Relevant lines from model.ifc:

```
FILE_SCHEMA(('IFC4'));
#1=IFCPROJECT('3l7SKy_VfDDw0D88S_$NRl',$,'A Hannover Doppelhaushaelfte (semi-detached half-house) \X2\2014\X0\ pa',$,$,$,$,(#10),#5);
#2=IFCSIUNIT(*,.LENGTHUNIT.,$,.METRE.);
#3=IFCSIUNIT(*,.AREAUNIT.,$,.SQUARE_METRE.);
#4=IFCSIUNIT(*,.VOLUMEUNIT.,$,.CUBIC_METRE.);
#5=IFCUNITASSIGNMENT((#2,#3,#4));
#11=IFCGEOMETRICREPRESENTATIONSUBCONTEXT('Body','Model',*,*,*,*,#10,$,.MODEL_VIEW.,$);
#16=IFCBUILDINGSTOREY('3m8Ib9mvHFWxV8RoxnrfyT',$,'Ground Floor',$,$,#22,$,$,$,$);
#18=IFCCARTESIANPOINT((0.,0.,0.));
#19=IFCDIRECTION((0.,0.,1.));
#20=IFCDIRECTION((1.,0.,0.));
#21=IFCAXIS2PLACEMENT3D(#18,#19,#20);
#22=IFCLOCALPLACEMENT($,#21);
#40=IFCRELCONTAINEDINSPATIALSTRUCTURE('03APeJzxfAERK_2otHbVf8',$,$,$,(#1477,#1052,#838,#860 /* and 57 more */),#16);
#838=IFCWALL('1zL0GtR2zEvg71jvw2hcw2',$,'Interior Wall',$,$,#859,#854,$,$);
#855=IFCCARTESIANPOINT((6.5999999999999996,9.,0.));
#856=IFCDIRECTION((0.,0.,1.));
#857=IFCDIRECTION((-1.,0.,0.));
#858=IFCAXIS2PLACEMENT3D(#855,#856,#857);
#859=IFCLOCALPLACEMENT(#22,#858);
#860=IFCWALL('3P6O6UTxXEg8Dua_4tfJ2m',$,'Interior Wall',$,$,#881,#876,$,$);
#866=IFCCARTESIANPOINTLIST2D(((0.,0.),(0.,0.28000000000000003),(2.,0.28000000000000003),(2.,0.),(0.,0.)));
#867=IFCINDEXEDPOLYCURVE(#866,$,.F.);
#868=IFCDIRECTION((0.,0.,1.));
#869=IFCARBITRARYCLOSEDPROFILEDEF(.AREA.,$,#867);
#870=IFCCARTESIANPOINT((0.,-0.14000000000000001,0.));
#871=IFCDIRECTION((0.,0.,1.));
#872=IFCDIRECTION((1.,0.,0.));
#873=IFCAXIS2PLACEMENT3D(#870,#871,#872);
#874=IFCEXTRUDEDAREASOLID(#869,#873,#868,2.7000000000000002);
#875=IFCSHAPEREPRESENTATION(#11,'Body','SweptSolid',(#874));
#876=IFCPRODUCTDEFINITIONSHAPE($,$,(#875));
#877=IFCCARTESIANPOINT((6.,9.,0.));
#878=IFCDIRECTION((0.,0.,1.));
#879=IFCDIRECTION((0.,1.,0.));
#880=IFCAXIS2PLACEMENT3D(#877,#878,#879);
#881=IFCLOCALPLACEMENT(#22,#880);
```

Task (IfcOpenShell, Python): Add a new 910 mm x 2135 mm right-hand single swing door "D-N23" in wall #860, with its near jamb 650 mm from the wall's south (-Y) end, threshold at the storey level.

```python
import numpy as np
import ifcopenshell
import ifcopenshell.api.feature
import ifcopenshell.api.geometry
import ifcopenshell.api.root
import ifcopenshell.api.spatial
import ifcopenshell.geom
import ifcopenshell.util.element
import ifcopenshell.util.placement
import ifcopenshell.util.representation
import ifcopenshell.util.shape
import ifcopenshell.util.unit

model = ifcopenshell.open("model.ifc")
unit_scale = ifcopenshell.util.unit.calculate_unit_scale(model)
settings = ifcopenshell.geom.settings()


def volume(element):
    """Net volume in cubic metres, openings subtracted."""
    shape = ifcopenshell.geom.create_shape(settings, element)
    return ifcopenshell.util.shape.get_volume(shape.geometry)


wall = model.by_guid("3P6O6UTxXEg8Dua_4tfJ2m")
storey = ifcopenshell.util.element.get_container(wall, ifc_class="IfcBuildingStorey")
context = ifcopenshell.util.representation.get_context(model, "Model", "Body", "MODEL_VIEW")
before = volume(wall)

width, height, from_end, sill = 0.91, 2.135, 0.65, 0.0  # metres

# The wall runs along its own X axis, and the end named is its -X end.
wall_shape = ifcopenshell.geom.create_shape(settings, wall)
x, y, z = ifcopenshell.util.shape.get_vertices(wall_shape.geometry).T
start = x.min() + from_end
face, thickness = float(y.min()), float(y.max() - y.min())
wall_matrix = ifcopenshell.util.placement.get_local_placement(wall.ObjectPlacement)
level = ifcopenshell.util.placement.get_local_placement(storey.ObjectPlacement)[2, 3]


def in_wall(x, y):
    """Placement at x, y metres in the wall's axes, at sill height."""
    matrix = wall_matrix.copy()
    matrix[:, 3] = wall_matrix @ np.array([x / unit_scale, y / unit_scale, 0.0, 1.0])
    matrix[2, 3] = level + sill / unit_scale
    return matrix


# Opening: a box that overshoots both wall faces by 50 mm.
opening = ifcopenshell.api.root.create_entity(model, ifc_class="IfcOpeningElement", predefined_type="OPENING")
box = ifcopenshell.api.geometry.add_wall_representation(
    model, context=context, length=width, height=height, thickness=thickness + 0.1
)
ifcopenshell.api.geometry.assign_representation(model, product=opening, representation=box)
ifcopenshell.api.geometry.edit_object_placement(model, product=opening, matrix=in_wall(start, face - 0.05), is_si=False)
ifcopenshell.api.feature.add_feature(model, feature=opening, element=wall)

door = ifcopenshell.api.root.create_entity(model, ifc_class="IfcDoor", name="D-N23", predefined_type="DOOR")
door.OverallWidth, door.OverallHeight = width / unit_scale, height / unit_scale
door.OperationType = "SINGLE_SWING_RIGHT"
body = ifcopenshell.api.geometry.add_door_representation(
    model,
    context=context,
    overall_width=door.OverallWidth,
    overall_height=door.OverallHeight,
    operation_type="SINGLE_SWING_RIGHT",
    lining_properties={"LiningDepth": thickness / unit_scale, "ThresholdDepth": thickness / unit_scale},
)
ifcopenshell.api.geometry.assign_representation(model, product=door, representation=body)
ifcopenshell.api.spatial.assign_container(model, products=[door], relating_structure=storey)
ifcopenshell.api.feature.add_filling(model, opening=opening, element=door)

# The lining spans the wall, so the door starts at the wall face.
ifcopenshell.api.geometry.edit_object_placement(model, product=door, matrix=in_wall(start, face), is_si=False)

after = volume(wall)

print(f"wall volume {before:.3f} -> {after:.3f} m3")

model.write("model_v2.ifc")
```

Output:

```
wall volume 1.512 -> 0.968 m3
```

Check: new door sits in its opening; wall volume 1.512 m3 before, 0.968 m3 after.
